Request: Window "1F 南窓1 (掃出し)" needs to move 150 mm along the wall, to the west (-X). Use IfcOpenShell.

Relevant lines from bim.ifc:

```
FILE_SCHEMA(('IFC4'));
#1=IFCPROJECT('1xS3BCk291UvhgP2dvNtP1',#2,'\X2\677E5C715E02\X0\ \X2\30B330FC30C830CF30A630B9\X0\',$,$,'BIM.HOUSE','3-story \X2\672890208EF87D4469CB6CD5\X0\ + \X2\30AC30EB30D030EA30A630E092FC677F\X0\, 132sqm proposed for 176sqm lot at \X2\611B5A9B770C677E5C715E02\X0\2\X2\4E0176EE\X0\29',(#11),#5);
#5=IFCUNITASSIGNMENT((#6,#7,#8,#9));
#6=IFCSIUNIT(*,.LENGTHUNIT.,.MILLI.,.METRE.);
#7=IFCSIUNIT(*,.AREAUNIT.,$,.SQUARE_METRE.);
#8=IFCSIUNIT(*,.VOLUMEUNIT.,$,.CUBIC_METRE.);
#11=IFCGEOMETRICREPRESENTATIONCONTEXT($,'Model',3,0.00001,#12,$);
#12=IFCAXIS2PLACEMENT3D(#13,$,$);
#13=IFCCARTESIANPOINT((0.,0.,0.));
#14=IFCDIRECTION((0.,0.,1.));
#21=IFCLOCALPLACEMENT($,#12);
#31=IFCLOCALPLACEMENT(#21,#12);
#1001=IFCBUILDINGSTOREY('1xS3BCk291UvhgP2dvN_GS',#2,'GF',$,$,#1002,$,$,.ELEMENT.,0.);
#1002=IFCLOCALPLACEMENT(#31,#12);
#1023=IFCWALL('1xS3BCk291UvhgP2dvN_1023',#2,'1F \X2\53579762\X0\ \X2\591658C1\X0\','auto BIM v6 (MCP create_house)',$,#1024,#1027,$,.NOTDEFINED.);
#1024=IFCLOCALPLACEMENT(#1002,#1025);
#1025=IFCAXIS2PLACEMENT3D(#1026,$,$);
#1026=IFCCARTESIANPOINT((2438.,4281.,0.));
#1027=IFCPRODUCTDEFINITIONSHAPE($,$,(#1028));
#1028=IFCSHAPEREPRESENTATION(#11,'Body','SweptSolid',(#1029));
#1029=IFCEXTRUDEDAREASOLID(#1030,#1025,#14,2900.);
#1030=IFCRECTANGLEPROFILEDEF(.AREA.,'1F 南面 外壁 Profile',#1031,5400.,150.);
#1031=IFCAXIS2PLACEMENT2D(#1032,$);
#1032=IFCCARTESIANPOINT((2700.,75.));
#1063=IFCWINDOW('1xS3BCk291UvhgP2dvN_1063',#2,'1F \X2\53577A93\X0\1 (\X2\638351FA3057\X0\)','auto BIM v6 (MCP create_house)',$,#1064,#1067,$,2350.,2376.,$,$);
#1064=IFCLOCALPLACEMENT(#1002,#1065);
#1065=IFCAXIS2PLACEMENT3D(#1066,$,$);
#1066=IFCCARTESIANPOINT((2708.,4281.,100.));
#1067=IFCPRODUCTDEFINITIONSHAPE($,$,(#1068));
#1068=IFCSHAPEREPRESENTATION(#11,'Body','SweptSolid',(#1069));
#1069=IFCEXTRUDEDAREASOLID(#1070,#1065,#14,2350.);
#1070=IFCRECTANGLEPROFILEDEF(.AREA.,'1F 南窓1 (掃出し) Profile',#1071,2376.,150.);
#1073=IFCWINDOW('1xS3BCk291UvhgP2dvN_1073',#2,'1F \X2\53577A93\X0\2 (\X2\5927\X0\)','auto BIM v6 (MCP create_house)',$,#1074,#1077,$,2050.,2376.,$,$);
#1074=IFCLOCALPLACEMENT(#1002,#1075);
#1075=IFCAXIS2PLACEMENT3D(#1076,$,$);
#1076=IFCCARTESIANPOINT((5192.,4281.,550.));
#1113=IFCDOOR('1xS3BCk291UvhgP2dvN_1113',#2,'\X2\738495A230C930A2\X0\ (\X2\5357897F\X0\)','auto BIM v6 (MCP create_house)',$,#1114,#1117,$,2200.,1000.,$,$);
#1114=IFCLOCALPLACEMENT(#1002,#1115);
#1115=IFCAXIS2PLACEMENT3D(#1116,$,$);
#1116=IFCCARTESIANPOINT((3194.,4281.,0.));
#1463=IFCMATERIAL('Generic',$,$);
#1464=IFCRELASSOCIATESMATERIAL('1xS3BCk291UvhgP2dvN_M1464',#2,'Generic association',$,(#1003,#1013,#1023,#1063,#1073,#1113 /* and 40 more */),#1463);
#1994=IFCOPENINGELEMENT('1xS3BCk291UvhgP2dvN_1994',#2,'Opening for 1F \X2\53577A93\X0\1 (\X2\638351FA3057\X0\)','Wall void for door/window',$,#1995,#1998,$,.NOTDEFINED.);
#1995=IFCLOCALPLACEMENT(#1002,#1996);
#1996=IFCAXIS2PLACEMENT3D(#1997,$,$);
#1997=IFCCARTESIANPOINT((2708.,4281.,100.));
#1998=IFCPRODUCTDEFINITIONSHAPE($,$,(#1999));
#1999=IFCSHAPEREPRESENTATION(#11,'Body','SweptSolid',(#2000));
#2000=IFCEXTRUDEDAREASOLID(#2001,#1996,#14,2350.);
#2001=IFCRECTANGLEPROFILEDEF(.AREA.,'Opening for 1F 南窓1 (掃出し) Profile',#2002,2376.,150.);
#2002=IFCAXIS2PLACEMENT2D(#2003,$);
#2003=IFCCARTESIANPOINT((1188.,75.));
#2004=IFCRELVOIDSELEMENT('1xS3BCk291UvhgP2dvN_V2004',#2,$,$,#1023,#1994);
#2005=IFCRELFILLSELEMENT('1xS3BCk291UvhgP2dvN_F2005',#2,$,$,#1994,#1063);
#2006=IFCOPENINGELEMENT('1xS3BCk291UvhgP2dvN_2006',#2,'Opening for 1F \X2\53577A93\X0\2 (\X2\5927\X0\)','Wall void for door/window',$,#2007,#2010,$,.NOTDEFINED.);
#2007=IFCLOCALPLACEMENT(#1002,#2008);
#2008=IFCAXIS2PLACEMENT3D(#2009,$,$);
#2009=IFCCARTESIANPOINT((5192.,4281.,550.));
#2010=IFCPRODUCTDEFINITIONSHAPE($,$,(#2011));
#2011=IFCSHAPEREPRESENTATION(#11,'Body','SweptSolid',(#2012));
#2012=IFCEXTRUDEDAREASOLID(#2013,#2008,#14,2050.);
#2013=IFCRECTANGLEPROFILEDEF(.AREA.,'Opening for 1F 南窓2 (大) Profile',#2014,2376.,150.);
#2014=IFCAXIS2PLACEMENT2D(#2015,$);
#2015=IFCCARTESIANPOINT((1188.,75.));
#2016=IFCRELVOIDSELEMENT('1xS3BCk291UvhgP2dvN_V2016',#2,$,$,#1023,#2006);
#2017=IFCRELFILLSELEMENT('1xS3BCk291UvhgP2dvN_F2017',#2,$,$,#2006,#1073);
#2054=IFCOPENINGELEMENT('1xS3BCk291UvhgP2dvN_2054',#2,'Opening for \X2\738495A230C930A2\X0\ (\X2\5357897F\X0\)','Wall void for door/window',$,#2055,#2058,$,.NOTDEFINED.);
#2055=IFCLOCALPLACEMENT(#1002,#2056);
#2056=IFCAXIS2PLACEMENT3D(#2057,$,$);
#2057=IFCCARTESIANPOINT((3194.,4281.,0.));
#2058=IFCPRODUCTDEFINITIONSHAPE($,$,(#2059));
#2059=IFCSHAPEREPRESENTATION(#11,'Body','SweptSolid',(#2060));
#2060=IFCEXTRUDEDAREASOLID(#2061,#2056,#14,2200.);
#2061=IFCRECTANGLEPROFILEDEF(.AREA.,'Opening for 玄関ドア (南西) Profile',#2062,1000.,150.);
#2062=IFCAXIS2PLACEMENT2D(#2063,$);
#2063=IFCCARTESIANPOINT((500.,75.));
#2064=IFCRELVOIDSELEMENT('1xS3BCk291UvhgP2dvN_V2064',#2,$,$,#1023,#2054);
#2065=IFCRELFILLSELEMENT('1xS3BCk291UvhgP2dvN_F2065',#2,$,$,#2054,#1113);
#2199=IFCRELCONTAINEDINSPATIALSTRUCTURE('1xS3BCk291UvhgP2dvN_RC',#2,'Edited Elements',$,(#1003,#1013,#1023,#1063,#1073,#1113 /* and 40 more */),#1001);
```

```python
import ifcopenshell
import ifcopenshell.api.geometry
import ifcopenshell.util.placement

model = ifcopenshell.open("bim.ifc")

window = model.by_guid("1xS3BCk291UvhgP2dvN_1063")
opening = window.FillsVoids[0].RelatingOpeningElement
wall = opening.VoidsElements[0].RelatingBuildingElement

wall_matrix = ifcopenshell.util.placement.get_local_placement(wall.ObjectPlacement)
shift = wall_matrix[:3, 0] * -150.0
before = ifcopenshell.util.placement.get_local_placement(window.ObjectPlacement)[:3, 3].copy()

# The window is not placed relative to its opening, so move both.
for product in (opening, window):
    matrix = ifcopenshell.util.placement.get_local_placement(product.ObjectPlacement)
    matrix[:3, 3] += shift
    ifcopenshell.api.geometry.edit_object_placement(model, product=product, matrix=matrix, is_si=False)

after = ifcopenshell.util.placement.get_local_placement(window.ObjectPlacement)[:3, 3]
print("window moved by", (after - before).round(3) + 0.0)

model.write("bim_rev.ifc")
```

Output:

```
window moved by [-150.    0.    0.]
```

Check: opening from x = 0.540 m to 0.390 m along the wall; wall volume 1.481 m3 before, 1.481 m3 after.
